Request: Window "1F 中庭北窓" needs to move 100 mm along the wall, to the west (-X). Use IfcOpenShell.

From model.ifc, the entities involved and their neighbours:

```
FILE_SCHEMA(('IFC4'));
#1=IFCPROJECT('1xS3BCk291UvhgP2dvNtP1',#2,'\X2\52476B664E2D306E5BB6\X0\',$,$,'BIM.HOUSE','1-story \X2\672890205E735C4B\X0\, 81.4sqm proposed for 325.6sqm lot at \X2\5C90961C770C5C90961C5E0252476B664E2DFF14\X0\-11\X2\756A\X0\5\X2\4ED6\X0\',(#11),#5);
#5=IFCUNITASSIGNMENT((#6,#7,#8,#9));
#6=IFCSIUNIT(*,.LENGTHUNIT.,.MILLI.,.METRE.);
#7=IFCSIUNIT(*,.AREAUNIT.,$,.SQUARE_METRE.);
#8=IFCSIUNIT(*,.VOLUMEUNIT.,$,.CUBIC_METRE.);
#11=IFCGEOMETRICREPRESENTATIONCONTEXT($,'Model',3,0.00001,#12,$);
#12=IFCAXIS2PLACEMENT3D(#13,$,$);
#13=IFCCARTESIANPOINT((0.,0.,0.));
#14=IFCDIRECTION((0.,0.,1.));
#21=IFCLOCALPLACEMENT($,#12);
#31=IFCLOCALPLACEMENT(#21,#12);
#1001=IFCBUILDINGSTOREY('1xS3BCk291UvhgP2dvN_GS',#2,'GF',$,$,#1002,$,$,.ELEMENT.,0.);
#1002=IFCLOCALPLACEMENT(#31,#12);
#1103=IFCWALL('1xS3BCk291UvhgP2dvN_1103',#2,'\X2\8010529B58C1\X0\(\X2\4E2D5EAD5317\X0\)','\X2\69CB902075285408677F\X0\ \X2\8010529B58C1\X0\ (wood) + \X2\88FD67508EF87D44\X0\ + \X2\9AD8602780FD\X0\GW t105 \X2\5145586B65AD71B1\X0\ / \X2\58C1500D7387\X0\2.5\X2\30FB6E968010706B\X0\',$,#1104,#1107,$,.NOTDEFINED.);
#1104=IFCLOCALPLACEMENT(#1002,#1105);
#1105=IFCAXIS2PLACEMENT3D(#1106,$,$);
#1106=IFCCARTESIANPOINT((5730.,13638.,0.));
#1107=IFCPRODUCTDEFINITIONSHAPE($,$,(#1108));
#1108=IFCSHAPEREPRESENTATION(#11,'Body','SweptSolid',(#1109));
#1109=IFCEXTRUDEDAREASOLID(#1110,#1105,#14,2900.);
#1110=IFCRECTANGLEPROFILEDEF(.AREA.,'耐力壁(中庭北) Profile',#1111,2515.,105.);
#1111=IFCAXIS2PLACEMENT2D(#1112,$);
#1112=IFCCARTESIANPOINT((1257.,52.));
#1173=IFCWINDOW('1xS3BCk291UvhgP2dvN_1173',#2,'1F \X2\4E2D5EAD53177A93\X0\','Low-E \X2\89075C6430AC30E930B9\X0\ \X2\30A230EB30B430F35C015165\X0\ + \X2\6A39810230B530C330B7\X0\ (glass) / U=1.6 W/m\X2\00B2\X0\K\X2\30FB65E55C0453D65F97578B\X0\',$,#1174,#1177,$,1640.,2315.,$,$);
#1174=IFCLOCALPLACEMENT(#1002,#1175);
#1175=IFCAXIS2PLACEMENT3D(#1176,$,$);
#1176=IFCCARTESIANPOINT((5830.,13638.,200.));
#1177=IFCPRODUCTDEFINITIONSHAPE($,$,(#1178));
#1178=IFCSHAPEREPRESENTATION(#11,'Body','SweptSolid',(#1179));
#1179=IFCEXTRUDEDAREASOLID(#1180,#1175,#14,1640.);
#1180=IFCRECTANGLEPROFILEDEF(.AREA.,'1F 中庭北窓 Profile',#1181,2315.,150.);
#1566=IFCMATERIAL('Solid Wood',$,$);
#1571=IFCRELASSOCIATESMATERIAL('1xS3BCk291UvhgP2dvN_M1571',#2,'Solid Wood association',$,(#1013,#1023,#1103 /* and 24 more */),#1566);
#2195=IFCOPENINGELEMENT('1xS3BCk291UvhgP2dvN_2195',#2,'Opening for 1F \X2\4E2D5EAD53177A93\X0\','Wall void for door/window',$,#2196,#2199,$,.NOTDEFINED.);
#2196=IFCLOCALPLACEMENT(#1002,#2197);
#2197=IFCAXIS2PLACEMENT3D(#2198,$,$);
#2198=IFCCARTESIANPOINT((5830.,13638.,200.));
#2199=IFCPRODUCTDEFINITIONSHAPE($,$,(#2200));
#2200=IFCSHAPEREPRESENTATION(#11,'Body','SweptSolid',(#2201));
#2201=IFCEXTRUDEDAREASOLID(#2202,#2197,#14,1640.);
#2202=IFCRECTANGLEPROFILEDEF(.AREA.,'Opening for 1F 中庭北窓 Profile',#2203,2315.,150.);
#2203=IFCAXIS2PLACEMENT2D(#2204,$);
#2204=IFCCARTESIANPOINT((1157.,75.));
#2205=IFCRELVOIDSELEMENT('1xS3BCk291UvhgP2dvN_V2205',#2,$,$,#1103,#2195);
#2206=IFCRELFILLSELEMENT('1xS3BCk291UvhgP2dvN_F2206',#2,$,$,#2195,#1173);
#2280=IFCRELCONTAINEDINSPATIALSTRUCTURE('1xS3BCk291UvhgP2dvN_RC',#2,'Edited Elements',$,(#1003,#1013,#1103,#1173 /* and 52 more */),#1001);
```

```python
import ifcopenshell
import ifcopenshell.api.geometry
import ifcopenshell.util.placement
import ifcopenshell.util.unit

model = ifcopenshell.open("model.ifc")
unit_scale = ifcopenshell.util.unit.calculate_unit_scale(model)

window = model.by_guid("1xS3BCk291UvhgP2dvN_1173")
opening = window.FillsVoids[0].RelatingOpeningElement
wall = opening.VoidsElements[0].RelatingBuildingElement

wall_matrix = ifcopenshell.util.placement.get_local_placement(wall.ObjectPlacement)
shift = wall_matrix[:3, 0] * -0.1 / unit_scale
before = ifcopenshell.util.placement.get_local_placement(window.ObjectPlacement)[:3, 3].copy()

# The window is not placed relative to its opening, so move both.
for product in (opening, window):
    matrix = ifcopenshell.util.placement.get_local_placement(product.ObjectPlacement)
    matrix[:3, 3] += shift
    ifcopenshell.api.geometry.edit_object_placement(model, product=product, matrix=matrix, is_si=False)

after = ifcopenshell.util.placement.get_local_placement(window.ObjectPlacement)[:3, 3]
print("window moved by", (after - before).round(3) + 0.0)

model.write("model_updated.ifc")
```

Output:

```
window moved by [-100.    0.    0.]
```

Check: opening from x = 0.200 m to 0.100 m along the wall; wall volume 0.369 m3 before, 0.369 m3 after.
